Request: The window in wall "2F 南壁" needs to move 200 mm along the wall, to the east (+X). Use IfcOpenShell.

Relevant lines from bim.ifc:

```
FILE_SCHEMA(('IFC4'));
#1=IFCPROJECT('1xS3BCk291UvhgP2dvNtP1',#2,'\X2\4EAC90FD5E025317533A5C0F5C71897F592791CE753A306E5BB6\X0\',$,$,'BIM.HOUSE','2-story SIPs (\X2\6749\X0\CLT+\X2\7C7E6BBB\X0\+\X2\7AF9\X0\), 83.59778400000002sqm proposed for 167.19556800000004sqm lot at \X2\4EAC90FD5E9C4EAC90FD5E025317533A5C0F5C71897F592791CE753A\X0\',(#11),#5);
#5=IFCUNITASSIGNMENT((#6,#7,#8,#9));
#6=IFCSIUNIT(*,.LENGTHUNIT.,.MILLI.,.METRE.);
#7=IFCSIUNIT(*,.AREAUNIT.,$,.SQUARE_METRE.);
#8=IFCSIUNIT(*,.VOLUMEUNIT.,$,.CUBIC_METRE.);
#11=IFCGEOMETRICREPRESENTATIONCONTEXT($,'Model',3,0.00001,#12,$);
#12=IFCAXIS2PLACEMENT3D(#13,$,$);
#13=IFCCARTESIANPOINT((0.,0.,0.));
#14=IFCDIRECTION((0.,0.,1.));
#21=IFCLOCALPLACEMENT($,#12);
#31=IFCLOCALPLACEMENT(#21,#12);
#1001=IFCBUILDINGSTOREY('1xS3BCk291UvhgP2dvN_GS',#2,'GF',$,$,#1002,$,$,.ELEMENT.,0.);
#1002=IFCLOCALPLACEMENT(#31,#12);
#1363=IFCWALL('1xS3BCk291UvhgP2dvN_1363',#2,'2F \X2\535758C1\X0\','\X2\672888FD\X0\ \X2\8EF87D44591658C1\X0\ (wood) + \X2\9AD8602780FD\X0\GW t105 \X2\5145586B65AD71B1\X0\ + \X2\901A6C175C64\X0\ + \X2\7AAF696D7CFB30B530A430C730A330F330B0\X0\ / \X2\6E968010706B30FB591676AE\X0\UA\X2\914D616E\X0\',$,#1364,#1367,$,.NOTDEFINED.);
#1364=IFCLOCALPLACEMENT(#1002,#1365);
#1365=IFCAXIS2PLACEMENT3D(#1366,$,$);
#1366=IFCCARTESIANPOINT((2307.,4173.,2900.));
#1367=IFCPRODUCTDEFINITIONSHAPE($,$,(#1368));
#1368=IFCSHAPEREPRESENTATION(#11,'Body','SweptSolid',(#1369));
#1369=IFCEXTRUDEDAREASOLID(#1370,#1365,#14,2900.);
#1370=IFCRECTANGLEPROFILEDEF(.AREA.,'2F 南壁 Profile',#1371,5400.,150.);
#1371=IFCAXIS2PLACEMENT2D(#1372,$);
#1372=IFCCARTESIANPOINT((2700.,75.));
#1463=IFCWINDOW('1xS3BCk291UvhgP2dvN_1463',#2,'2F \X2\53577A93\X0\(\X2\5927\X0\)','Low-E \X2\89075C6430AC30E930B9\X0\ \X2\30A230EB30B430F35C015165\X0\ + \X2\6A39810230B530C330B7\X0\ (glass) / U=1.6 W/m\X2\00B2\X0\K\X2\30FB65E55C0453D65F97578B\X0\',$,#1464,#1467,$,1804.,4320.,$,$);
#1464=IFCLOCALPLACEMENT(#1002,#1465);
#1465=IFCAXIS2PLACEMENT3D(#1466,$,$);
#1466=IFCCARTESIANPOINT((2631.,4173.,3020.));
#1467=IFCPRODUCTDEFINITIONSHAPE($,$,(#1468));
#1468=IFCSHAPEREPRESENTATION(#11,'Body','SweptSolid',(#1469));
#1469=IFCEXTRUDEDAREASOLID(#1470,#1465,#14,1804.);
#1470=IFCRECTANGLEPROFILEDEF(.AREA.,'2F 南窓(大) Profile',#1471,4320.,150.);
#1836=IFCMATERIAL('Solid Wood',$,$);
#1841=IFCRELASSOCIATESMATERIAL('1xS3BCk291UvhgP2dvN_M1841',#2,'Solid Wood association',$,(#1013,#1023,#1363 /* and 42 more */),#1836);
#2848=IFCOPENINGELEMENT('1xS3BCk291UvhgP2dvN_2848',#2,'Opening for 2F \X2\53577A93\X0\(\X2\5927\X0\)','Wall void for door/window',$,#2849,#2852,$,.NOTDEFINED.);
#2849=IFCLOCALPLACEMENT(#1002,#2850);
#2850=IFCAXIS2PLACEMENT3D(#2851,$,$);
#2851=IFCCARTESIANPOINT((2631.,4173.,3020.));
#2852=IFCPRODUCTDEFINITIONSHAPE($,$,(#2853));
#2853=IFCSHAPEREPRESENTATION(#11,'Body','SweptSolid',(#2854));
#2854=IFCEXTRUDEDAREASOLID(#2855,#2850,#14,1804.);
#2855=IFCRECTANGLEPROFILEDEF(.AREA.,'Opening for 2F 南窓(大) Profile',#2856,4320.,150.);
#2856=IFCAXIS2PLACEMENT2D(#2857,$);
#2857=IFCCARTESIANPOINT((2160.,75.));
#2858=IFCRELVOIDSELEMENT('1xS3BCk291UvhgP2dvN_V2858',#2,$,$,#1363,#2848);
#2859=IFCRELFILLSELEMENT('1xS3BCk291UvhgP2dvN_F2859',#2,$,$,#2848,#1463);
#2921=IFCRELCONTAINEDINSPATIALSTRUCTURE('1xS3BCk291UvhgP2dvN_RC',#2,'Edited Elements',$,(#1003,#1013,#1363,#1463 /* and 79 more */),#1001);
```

```python
import ifcopenshell
import ifcopenshell.api.geometry
import ifcopenshell.util.placement
import ifcopenshell.util.unit

model = ifcopenshell.open("bim.ifc")
unit_scale = ifcopenshell.util.unit.calculate_unit_scale(model)

window = model.by_guid("1xS3BCk291UvhgP2dvN_1463")
opening = window.FillsVoids[0].RelatingOpeningElement
wall = opening.VoidsElements[0].RelatingBuildingElement

wall_matrix = ifcopenshell.util.placement.get_local_placement(wall.ObjectPlacement)
shift = wall_matrix[:3, 0] * 0.2 / unit_scale
before = ifcopenshell.util.placement.get_local_placement(window.ObjectPlacement)[:3, 3].copy()

# The window is not placed relative to its opening, so move both.
for product in (opening, window):
    matrix = ifcopenshell.util.placement.get_local_placement(product.ObjectPlacement)
    matrix[:3, 3] += shift
    ifcopenshell.api.geometry.edit_object_placement(model, product=product, matrix=matrix, is_si=False)

after = ifcopenshell.util.placement.get_local_placement(window.ObjectPlacement)[:3, 3]
print("window moved by", (after - before).round(3) + 0.0)

model.write("bim-out.ifc")
```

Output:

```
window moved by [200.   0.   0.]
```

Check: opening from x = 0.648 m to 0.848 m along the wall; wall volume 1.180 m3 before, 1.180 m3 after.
